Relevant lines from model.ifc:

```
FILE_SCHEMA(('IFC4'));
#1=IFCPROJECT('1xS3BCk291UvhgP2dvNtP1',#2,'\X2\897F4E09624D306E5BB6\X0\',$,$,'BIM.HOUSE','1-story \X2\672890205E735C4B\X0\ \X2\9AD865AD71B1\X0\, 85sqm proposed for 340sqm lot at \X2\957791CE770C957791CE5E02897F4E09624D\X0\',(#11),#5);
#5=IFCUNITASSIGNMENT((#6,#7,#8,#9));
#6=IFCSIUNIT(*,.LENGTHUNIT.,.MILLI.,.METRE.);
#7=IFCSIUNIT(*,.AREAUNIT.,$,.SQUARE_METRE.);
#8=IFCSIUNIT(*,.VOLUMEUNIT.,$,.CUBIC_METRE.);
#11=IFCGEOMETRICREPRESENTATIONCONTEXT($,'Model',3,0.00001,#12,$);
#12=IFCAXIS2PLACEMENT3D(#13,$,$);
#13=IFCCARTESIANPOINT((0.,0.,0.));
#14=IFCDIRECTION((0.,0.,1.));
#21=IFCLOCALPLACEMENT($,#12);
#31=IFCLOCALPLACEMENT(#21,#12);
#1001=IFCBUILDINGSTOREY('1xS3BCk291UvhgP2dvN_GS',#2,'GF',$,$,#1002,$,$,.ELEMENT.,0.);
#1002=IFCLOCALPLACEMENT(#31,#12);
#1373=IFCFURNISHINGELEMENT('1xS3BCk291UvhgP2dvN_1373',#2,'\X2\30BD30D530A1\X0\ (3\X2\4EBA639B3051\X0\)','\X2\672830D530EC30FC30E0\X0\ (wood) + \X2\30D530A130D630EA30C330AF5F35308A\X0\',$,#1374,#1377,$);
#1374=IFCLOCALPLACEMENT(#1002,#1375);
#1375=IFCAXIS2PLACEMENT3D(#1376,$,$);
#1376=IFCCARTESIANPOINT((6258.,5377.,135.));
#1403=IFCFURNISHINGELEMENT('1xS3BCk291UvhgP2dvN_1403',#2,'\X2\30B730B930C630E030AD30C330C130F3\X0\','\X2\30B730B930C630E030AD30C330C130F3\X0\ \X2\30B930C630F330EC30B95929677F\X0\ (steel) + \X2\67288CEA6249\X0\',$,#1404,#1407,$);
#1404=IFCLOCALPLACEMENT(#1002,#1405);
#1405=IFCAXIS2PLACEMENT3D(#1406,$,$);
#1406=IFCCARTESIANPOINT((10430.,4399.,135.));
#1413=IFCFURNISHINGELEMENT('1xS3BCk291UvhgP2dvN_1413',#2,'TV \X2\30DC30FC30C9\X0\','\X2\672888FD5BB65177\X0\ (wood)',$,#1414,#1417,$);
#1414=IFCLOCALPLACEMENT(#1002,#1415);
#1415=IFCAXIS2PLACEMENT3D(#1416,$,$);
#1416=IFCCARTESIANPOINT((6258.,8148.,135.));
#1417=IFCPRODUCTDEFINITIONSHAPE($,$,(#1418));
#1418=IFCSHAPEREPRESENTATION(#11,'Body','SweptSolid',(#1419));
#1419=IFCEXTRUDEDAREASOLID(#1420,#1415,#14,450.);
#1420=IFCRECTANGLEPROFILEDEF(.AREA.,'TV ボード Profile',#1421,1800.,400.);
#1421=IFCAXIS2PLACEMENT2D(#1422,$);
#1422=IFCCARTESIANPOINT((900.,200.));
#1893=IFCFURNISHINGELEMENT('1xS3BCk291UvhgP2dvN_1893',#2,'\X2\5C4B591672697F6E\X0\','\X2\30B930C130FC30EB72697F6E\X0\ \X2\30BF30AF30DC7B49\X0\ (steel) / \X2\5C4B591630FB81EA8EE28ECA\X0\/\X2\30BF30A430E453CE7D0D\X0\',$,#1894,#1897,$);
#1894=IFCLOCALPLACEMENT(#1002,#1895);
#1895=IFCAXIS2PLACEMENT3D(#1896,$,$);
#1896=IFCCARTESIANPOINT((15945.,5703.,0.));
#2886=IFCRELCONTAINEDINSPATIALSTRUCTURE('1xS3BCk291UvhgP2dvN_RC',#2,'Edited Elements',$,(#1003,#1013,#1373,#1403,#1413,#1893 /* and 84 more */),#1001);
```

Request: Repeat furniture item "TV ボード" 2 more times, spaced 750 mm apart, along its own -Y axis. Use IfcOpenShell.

```python
import ifcopenshell
import ifcopenshell.api.geometry
import ifcopenshell.api.root
import ifcopenshell.util.element
import ifcopenshell.util.placement
import ifcopenshell.util.unit

model = ifcopenshell.open("model.ifc")
unit_scale = ifcopenshell.util.unit.calculate_unit_scale(model)


def reuse_history(source, copy):
    """copy_class also copies each property set's owner history, people and application; keep the originals."""
    for rel in copy.IsDefinedBy:
        if rel.is_a("IfcRelDefinesByProperties") and (history := rel.RelatingPropertyDefinition.OwnerHistory):
            rel.RelatingPropertyDefinition.OwnerHistory = source.OwnerHistory
            ifcopenshell.util.element.remove_deep2(model, history)


source = model.by_id(1413)
base = ifcopenshell.util.placement.get_local_placement(source.ObjectPlacement)
step = -base[:3, 1] * 0.75 / unit_scale

for i in range(1, 3):
    copy = ifcopenshell.api.root.copy_class(model, product=source)
    copy.Representation = ifcopenshell.util.element.copy_deep(
        model, source.Representation, exclude=["IfcGeometricRepresentationContext", "IfcRepresentationMap"]
    )
    reuse_history(source, copy)
    matrix = base.copy()
    matrix[:3, 3] += i * step
    print("added at", matrix[:3, 3].round(3) + 0.0)
    ifcopenshell.api.geometry.edit_object_placement(model, product=copy, matrix=matrix, is_si=False)

model.write("model_updated.ifc")
```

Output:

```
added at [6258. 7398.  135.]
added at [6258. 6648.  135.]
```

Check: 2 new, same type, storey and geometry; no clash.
